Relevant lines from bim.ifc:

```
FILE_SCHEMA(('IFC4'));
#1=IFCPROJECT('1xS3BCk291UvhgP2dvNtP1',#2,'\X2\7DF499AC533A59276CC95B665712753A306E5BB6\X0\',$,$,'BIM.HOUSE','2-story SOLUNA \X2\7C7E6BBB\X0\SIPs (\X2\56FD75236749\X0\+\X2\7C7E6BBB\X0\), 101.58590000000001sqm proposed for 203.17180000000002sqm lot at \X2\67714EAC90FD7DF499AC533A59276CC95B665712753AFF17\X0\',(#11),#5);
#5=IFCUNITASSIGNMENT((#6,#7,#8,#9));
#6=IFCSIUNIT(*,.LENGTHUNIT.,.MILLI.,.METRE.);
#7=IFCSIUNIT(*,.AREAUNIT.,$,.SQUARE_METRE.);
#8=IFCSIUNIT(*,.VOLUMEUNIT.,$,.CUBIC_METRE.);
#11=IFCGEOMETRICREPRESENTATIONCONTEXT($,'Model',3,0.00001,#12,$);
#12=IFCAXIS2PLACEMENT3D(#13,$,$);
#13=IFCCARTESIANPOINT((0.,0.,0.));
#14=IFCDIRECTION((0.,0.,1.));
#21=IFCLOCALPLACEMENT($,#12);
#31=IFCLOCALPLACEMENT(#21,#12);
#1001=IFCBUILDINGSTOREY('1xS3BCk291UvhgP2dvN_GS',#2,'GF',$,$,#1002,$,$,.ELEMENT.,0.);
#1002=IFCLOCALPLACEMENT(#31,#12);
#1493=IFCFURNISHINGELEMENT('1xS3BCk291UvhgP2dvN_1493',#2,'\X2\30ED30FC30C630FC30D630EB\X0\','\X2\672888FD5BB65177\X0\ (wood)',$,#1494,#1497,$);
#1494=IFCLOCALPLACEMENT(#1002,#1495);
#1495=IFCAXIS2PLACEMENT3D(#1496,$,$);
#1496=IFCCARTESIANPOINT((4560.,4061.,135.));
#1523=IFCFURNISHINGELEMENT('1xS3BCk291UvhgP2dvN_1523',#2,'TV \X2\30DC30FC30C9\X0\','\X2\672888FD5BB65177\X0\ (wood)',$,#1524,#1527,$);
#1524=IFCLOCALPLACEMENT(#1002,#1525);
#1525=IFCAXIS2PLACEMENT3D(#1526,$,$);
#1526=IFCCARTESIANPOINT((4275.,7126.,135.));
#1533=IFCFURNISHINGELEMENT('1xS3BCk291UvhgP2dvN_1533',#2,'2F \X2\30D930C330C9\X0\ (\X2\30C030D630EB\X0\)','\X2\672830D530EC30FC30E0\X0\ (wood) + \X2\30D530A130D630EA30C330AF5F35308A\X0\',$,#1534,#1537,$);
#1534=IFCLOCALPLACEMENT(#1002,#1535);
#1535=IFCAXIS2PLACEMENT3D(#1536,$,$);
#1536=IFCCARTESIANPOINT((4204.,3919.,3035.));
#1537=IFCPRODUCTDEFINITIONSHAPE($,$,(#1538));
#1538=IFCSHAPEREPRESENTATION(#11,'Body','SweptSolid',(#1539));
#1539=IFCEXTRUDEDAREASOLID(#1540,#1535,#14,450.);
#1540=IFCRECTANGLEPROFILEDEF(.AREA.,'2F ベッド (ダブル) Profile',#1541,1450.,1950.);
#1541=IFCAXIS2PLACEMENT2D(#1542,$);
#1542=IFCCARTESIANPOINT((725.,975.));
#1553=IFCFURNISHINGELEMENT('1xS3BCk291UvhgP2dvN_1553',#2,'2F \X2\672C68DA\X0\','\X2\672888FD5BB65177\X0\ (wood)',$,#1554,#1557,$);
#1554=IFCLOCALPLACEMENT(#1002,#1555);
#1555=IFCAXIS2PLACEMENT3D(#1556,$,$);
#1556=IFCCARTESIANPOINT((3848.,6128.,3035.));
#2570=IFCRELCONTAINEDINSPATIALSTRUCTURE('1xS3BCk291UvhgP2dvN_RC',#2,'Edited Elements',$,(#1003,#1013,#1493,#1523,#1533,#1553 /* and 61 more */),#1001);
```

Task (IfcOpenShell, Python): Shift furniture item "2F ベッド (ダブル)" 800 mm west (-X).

```python
import ifcopenshell
import ifcopenshell.api.geometry
import ifcopenshell.util.placement
import ifcopenshell.util.unit

model = ifcopenshell.open("bim.ifc")
unit_scale = ifcopenshell.util.unit.calculate_unit_scale(model)

item = model.by_guid("1xS3BCk291UvhgP2dvN_1533")
matrix = ifcopenshell.util.placement.get_local_placement(item.ObjectPlacement)
matrix[0, 3] -= 0.8 / unit_scale
ifcopenshell.api.geometry.edit_object_placement(model, product=item, matrix=matrix, is_si=False)

print(ifcopenshell.util.placement.get_local_placement(item.ObjectPlacement).round(3) + 0.0)

model.write("bim_updated.ifc")
```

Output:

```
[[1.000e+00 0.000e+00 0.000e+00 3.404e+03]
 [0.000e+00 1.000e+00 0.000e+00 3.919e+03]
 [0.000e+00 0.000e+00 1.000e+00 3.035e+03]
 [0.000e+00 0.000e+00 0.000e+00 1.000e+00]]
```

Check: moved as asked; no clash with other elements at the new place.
